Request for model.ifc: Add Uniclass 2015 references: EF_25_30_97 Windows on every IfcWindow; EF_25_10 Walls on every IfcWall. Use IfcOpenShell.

First a look at what the model holds.

```python
import ifcopenshell

model = ifcopenshell.open("model.ifc")
print(model.schema)
print("classifications:", [c.Name for c in model.by_type("IfcClassification")])
for ifc_class in ("IfcDoor", "IfcRoof", "IfcStair", "IfcWall", "IfcWindow"):
    print(ifc_class, len(model.by_type(ifc_class)))
```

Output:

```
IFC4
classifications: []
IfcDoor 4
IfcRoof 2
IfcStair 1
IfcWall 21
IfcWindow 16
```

```python
import ifcopenshell
import ifcopenshell.api.classification

model = ifcopenshell.open("model.ifc")

system = ifcopenshell.api.classification.add_classification(model, classification="Uniclass 2015")

codes = {
    "IfcWindow": ("EF_25_30_97", "Windows"),
    "IfcWall": ("EF_25_10", "Walls"),
}
for ifc_class, (code, name) in codes.items():
    products = model.by_type(ifc_class)
    ifcopenshell.api.classification.add_reference(
        model, products=products, classification=system, identification=code, name=name
    )
    print(code, len(products))

model.write("model_edited.ifc")
```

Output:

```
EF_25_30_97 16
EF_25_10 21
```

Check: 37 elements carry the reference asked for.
